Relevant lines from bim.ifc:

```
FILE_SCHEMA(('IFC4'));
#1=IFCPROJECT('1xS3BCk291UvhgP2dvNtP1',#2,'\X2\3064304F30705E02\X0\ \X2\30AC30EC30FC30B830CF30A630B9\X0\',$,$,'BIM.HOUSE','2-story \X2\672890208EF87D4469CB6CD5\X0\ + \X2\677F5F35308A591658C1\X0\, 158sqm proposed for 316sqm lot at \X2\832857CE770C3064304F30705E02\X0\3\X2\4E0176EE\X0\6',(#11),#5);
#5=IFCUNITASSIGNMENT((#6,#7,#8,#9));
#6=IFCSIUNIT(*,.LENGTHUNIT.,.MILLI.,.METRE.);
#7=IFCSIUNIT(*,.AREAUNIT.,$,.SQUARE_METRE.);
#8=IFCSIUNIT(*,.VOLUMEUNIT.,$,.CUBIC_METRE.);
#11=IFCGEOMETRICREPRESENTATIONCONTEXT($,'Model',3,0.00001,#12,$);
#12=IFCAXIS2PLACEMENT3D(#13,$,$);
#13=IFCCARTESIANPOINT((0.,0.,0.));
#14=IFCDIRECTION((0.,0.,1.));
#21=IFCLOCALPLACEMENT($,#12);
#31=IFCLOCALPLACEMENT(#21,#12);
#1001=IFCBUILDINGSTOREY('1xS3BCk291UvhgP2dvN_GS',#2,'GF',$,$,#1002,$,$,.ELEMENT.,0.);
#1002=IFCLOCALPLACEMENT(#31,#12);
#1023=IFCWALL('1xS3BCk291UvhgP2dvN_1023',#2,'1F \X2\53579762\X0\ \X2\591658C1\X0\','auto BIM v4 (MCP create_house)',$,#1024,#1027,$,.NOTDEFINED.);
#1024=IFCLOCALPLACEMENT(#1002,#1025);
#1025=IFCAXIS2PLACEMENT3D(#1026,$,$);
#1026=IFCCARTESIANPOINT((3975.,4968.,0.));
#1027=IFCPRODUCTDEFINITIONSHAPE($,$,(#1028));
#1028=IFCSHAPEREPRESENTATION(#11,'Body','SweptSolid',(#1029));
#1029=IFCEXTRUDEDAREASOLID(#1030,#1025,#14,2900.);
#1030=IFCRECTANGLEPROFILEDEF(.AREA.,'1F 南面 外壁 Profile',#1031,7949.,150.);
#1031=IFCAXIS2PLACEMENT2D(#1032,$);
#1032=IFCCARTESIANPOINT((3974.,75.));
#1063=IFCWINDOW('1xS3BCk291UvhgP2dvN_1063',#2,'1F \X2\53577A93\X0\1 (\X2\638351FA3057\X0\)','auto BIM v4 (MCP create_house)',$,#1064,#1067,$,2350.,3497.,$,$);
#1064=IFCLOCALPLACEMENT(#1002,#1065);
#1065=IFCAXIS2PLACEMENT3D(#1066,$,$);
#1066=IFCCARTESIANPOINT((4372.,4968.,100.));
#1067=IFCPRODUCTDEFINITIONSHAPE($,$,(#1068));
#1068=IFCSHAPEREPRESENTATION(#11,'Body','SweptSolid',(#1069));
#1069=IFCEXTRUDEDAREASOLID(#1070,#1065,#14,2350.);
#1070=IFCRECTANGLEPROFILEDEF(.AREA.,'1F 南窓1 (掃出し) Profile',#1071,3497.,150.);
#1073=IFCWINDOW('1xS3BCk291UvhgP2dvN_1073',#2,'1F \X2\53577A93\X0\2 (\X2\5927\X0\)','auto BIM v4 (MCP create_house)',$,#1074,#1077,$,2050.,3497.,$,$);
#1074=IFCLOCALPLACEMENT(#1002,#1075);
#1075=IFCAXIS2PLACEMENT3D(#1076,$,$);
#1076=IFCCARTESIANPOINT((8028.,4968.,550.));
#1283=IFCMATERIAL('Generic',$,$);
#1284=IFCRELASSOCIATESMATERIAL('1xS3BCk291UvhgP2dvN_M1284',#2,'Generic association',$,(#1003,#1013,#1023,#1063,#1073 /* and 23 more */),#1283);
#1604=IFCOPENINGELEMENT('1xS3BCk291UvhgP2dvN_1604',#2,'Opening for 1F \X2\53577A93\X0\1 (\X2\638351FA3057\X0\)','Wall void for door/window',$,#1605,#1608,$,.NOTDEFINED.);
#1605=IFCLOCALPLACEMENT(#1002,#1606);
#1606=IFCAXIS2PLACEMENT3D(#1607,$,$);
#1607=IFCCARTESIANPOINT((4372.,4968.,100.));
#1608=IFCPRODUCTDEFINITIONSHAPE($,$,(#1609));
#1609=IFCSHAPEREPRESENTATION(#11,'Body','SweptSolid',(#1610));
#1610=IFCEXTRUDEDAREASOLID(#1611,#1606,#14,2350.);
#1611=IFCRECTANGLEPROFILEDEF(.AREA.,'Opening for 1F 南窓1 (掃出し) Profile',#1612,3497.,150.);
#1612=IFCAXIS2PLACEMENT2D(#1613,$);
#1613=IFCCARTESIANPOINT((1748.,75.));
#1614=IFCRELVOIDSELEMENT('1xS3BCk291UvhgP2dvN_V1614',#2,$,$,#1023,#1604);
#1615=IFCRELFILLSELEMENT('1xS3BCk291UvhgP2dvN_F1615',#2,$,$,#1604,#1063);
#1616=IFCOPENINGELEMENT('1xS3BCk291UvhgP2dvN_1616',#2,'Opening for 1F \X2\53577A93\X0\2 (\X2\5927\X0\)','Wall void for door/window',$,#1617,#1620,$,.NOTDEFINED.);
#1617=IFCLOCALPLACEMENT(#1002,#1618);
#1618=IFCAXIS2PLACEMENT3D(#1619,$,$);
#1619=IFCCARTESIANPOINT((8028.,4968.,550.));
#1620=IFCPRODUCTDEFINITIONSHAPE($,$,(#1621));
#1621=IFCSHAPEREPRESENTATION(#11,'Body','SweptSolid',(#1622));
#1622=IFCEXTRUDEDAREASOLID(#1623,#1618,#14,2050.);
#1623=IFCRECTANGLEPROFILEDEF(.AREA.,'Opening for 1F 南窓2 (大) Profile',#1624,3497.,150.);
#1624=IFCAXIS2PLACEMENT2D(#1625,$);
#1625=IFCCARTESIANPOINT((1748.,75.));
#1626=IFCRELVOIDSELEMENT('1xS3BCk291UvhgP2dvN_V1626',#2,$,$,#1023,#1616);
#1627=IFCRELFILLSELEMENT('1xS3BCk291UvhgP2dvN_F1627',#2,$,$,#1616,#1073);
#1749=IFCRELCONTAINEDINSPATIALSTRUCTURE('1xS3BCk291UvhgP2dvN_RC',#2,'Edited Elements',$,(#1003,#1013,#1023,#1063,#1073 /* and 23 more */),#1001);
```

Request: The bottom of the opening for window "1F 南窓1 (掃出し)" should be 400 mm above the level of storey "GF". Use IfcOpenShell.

```python
import numpy as np
import ifcopenshell
import ifcopenshell.api.geometry
import ifcopenshell.geom
import ifcopenshell.util.element
import ifcopenshell.util.placement
import ifcopenshell.util.shape
import ifcopenshell.util.unit

model = ifcopenshell.open("bim.ifc")
unit_scale = ifcopenshell.util.unit.calculate_unit_scale(model)

window = model.by_guid("1xS3BCk291UvhgP2dvN_1063")
opening = window.FillsVoids[0].RelatingOpeningElement
storey = ifcopenshell.util.element.get_container(window, ifc_class="IfcBuildingStorey")
level = ifcopenshell.util.placement.get_local_placement(storey.ObjectPlacement)[2, 3]

# The opening's origin need not be at the sill, so measure its lowest point.
shape = ifcopenshell.geom.create_shape(ifcopenshell.geom.settings(), opening)
bottom = ifcopenshell.util.shape.get_shape_bottom_elevation(shape, shape.geometry) / unit_scale
dz = level + 0.4 / unit_scale - bottom

shift = np.array([0.0, 0.0, dz])
# The window is not placed relative to its opening, so move both.
for product in (opening, window):
    matrix = ifcopenshell.util.placement.get_local_placement(product.ObjectPlacement)
    matrix[:3, 3] += shift
    ifcopenshell.api.geometry.edit_object_placement(model, product=product, matrix=matrix, is_si=False)

print(f"moved by {dz * unit_scale:+.3f} m")

model.write("bim_v2.ifc")
```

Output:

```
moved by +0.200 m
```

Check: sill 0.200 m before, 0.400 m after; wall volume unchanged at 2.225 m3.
